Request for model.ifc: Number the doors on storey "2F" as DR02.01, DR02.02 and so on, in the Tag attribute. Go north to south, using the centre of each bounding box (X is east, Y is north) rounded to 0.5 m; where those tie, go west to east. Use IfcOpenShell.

First a look at what the model holds.

```python
import ifcopenshell
import ifcopenshell.util.element
import ifcopenshell.util.placement

model = ifcopenshell.open("model.ifc")
print(model.schema)
storey = next(s for s in model.by_type("IfcBuildingStorey") if s.Name == "2F")
doors = [e for e in ifcopenshell.util.element.get_decomposition(storey) if e.is_a("IfcDoor")]
for e in sorted(doors, key=lambda e: e.id()):
    origin = ifcopenshell.util.placement.get_local_placement(e.ObjectPlacement)[:3, 3]
    print(e.id(), e.Tag, e.Name, origin.round(2) + 0.0, sep=" | ")
```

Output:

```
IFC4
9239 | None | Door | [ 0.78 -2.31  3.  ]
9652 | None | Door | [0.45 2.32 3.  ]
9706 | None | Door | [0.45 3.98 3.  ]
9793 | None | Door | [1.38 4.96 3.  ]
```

```python
import ifcopenshell
import ifcopenshell.geom
import ifcopenshell.util.element
import ifcopenshell.util.shape

model = ifcopenshell.open("model.ifc")
settings = ifcopenshell.geom.settings()
settings.set("use-world-coords", True)


def centre(element):
    shape = ifcopenshell.geom.create_shape(settings, element)
    return ifcopenshell.util.shape.get_bbox_centroid(shape.geometry)


storey = next(s for s in model.by_type("IfcBuildingStorey") if s.Name == "2F")
doors = [e for e in ifcopenshell.util.element.get_decomposition(storey) if e.is_a("IfcDoor")]

# Insertion points can sit at a corner or the storey origin, so sort by the geometry (in metres).
centres = {e: centre(e) for e in doors}
doors.sort(key=lambda e: (-round(centres[e][1] / 0.5), centres[e][0]))

for i, e in enumerate(doors, start=1):
    number = f"DR02.{i:02d}"
    e.Tag = number
    print(e.id(), number)

model.write("model_updated.ifc")
```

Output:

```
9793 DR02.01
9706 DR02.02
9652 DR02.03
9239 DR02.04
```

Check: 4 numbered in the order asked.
